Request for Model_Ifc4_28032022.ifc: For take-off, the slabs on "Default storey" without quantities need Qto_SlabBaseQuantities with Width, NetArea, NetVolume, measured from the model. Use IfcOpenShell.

First a look at what the model holds.

```python
import ifcopenshell
import ifcopenshell.util.element
import ifcopenshell.util.unit

model = ifcopenshell.open("Model_Ifc4_28032022.ifc")
print(model.schema)
for unit_type in ("LENGTHUNIT", "AREAUNIT", "VOLUMEUNIT"):
    print(unit_type, ifcopenshell.util.unit.calculate_unit_scale(model, unit_type))
storey = next(s for s in model.by_type("IfcBuildingStorey") if s.Name == "Default storey")
slabs = [e for e in ifcopenshell.util.element.get_decomposition(storey) if e.is_a("IfcSlab")]
for e in sorted(slabs, key=lambda e: e.id()):
    print(e.id(), e.is_a(), e.Name, list(ifcopenshell.util.element.get_psets(e, qtos_only=True)), sep=" | ")
```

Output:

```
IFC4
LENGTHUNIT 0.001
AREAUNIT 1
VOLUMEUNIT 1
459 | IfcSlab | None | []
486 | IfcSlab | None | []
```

```python
import ifcopenshell
import ifcopenshell.api.pset
import ifcopenshell.geom
import ifcopenshell.util.element
import ifcopenshell.util.shape
import ifcopenshell.util.unit

model = ifcopenshell.open("Model_Ifc4_28032022.ifc")
unit_scale = ifcopenshell.util.unit.calculate_unit_scale(model)
area_scale = ifcopenshell.util.unit.calculate_unit_scale(model, "AREAUNIT")
volume_scale = ifcopenshell.util.unit.calculate_unit_scale(model, "VOLUMEUNIT")
settings = ifcopenshell.geom.settings()

storey = next(s for s in model.by_type("IfcBuildingStorey") if s.Name == "Default storey")
slabs = [e for e in ifcopenshell.util.element.get_decomposition(storey) if e.is_a("IfcSlab")]

for e in sorted(slabs, key=lambda e: e.id()):
    if ifcopenshell.util.element.get_psets(e, qtos_only=True, should_inherit=False):
        continue
    # Geometry comes back in metres, in the element's own axes.
    shape = ifcopenshell.geom.create_shape(settings, e)
    values = {
        "Width": ifcopenshell.util.shape.get_z(shape.geometry) / unit_scale,
        "NetArea": ifcopenshell.util.shape.get_footprint_area(shape.geometry) / area_scale,
        "NetVolume": ifcopenshell.util.shape.get_volume(shape.geometry) / volume_scale,
    }
    qto = ifcopenshell.api.pset.add_qto(model, product=e, name="Qto_SlabBaseQuantities")
    ifcopenshell.api.pset.edit_qto(model, qto=qto, properties=values)
    print(e.id(), {k: round(v, 3) for k, v in values.items()})

model.write("Model_Ifc4_28032022_edited.ifc")
```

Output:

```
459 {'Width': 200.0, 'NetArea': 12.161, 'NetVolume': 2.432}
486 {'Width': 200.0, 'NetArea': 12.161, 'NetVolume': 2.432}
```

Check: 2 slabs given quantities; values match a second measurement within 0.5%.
